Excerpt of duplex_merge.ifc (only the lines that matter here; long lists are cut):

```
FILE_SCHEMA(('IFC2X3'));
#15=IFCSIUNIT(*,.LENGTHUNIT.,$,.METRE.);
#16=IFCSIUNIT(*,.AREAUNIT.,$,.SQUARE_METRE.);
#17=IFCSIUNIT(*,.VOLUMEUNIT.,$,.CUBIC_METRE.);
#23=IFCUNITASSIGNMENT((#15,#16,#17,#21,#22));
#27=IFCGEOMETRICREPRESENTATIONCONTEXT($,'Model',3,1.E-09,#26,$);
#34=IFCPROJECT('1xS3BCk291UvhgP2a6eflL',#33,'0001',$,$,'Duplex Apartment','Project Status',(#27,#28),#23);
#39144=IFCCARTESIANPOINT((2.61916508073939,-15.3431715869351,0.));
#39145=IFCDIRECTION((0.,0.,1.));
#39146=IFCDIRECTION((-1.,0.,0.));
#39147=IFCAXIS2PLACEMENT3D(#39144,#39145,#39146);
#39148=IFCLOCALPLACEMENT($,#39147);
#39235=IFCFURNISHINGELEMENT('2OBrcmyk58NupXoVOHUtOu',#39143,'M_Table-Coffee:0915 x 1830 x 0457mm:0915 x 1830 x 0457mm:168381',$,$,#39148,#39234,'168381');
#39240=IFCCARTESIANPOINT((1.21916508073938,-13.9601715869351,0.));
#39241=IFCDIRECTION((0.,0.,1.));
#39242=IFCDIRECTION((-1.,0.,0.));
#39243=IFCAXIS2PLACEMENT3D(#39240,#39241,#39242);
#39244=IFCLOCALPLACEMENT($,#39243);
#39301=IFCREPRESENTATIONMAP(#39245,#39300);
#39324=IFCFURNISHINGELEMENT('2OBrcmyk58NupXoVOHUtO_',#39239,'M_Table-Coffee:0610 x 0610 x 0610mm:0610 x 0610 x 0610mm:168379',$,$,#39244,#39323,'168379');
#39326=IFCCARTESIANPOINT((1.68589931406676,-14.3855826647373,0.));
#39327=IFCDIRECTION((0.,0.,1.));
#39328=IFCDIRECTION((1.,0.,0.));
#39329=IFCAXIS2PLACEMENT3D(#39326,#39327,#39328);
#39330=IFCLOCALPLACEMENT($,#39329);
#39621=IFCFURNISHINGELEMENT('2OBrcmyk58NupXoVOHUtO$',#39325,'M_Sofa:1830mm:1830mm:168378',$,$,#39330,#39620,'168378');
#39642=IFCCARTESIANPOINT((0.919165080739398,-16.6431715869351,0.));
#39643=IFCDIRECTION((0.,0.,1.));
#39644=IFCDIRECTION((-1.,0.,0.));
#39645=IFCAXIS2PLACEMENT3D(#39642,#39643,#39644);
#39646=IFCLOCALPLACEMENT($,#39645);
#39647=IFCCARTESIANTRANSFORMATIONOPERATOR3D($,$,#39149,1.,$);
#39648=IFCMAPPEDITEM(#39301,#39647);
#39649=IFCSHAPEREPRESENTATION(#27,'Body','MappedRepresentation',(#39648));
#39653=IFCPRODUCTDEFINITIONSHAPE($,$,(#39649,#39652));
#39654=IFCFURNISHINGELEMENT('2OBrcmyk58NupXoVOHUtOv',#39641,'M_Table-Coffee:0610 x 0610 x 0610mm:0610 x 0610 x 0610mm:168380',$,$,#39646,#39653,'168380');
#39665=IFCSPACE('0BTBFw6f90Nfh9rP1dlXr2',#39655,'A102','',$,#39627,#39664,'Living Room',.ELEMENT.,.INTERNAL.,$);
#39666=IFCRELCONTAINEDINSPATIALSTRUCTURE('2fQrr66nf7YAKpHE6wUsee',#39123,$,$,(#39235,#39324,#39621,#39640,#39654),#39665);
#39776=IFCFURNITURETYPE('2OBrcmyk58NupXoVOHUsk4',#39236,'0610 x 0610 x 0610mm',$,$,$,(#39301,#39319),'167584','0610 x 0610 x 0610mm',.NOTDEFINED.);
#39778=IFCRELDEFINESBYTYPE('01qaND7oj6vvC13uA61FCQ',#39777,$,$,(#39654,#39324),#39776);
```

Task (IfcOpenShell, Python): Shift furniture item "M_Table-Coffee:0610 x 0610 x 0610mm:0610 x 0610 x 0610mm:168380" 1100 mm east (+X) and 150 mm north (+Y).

```python
import ifcopenshell
import ifcopenshell.api.geometry
import ifcopenshell.util.placement
import ifcopenshell.util.unit

model = ifcopenshell.open("duplex_merge.ifc")
unit_scale = ifcopenshell.util.unit.calculate_unit_scale(model)

item = model.by_guid("2OBrcmyk58NupXoVOHUtOv")
matrix = ifcopenshell.util.placement.get_local_placement(item.ObjectPlacement)
matrix[0, 3] += 1.1 / unit_scale
matrix[1, 3] += 0.15 / unit_scale
ifcopenshell.api.geometry.edit_object_placement(model, product=item, matrix=matrix, is_si=False)

print(ifcopenshell.util.placement.get_local_placement(item.ObjectPlacement).round(3) + 0.0)

model.write("duplex_merge_updated.ifc")
```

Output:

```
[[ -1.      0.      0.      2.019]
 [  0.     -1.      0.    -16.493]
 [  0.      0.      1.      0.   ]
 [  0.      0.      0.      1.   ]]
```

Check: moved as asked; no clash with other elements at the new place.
